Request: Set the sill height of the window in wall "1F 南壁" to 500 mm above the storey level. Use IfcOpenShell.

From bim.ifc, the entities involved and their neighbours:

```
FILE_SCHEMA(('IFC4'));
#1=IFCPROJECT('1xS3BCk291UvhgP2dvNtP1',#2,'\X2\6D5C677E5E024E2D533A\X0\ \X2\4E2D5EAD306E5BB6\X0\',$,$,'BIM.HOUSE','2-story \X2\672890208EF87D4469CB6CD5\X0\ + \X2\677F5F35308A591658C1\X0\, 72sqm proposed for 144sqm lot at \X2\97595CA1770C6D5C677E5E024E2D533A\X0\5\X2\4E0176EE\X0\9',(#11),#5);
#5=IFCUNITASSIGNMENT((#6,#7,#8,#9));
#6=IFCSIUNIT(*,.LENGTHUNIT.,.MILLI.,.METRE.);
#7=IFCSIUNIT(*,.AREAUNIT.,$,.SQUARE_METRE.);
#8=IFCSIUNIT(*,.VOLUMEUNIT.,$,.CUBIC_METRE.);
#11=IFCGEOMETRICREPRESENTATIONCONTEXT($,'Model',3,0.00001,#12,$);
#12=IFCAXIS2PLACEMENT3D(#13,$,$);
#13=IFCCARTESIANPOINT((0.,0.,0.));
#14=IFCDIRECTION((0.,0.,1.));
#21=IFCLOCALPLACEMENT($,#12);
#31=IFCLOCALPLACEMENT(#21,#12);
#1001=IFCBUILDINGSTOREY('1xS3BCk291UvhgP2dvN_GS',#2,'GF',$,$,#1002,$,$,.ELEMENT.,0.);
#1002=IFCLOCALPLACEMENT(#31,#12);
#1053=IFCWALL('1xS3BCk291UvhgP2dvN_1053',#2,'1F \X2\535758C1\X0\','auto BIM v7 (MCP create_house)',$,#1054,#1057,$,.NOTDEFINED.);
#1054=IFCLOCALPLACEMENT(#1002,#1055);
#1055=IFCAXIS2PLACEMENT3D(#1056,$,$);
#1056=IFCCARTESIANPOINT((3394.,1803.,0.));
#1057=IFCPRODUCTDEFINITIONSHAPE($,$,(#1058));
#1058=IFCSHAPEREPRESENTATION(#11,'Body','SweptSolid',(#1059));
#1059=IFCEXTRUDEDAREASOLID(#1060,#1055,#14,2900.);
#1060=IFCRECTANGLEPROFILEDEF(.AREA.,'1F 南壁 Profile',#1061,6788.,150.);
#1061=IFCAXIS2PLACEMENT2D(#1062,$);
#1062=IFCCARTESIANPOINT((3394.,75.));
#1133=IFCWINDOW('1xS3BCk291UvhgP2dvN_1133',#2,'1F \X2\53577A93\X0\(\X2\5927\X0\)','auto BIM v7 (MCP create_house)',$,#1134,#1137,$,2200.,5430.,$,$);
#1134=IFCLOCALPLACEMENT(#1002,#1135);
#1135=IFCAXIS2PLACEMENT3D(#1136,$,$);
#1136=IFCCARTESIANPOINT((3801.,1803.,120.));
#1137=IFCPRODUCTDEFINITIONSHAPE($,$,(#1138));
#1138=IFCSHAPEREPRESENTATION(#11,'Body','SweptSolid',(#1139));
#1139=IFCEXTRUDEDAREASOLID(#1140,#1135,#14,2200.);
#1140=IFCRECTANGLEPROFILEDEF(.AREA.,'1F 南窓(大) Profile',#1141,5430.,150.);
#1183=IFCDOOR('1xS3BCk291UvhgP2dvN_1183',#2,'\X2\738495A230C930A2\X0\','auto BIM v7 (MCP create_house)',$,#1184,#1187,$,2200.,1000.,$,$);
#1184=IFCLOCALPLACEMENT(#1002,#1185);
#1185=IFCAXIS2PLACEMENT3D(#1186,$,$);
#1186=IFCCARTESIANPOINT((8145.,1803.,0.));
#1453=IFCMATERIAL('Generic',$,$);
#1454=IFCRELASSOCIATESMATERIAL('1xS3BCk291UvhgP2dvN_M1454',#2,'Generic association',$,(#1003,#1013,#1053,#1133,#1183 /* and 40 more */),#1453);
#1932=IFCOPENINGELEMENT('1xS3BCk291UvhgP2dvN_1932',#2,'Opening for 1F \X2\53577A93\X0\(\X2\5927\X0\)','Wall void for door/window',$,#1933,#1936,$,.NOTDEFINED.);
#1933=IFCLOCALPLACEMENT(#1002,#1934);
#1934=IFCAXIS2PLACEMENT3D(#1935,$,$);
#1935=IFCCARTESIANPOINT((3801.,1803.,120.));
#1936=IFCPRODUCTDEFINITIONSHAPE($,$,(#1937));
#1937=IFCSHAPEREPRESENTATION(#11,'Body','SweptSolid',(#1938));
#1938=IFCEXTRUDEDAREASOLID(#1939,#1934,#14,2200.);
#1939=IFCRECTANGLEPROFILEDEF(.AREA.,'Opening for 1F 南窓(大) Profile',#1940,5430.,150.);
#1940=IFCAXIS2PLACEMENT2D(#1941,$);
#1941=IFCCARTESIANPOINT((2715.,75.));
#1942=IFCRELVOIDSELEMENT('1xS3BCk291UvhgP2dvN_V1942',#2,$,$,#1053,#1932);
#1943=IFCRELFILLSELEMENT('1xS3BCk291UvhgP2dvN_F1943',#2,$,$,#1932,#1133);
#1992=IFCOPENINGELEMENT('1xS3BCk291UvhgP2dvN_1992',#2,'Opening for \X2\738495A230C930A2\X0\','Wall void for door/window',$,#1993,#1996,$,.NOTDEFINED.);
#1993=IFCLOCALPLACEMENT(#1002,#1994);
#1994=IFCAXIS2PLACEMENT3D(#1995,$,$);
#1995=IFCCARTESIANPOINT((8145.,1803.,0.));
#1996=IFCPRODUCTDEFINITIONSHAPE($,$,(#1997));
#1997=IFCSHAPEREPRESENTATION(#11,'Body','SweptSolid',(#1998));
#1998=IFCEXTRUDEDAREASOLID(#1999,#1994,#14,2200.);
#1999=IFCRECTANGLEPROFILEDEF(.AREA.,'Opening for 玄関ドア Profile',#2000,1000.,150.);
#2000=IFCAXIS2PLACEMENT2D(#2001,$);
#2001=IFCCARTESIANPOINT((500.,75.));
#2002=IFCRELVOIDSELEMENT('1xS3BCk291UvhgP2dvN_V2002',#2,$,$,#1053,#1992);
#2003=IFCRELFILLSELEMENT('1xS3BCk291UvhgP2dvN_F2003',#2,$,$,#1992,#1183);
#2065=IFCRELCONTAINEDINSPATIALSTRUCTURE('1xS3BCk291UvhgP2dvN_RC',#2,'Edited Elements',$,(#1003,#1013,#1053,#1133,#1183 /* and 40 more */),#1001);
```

```python
import numpy as np
import ifcopenshell
import ifcopenshell.api.geometry
import ifcopenshell.geom
import ifcopenshell.util.element
import ifcopenshell.util.placement
import ifcopenshell.util.shape
import ifcopenshell.util.unit

model = ifcopenshell.open("bim.ifc")
unit_scale = ifcopenshell.util.unit.calculate_unit_scale(model)

window = model.by_guid("1xS3BCk291UvhgP2dvN_1133")
opening = window.FillsVoids[0].RelatingOpeningElement
storey = ifcopenshell.util.element.get_container(window, ifc_class="IfcBuildingStorey")
level = ifcopenshell.util.placement.get_local_placement(storey.ObjectPlacement)[2, 3]

# The opening's origin need not be at the sill, so measure its lowest point.
shape = ifcopenshell.geom.create_shape(ifcopenshell.geom.settings(), opening)
bottom = ifcopenshell.util.shape.get_shape_bottom_elevation(shape, shape.geometry) / unit_scale
dz = level + 500.0 - bottom

shift = np.array([0.0, 0.0, dz])
# The window is not placed relative to its opening, so move both.
for product in (opening, window):
    matrix = ifcopenshell.util.placement.get_local_placement(product.ObjectPlacement)
    matrix[:3, 3] += shift
    ifcopenshell.api.geometry.edit_object_placement(model, product=product, matrix=matrix, is_si=False)

print(f"moved by {dz * unit_scale:+.3f} m")

model.write("bim_edited.ifc")
```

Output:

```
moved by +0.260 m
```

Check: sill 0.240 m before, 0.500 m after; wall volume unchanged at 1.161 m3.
